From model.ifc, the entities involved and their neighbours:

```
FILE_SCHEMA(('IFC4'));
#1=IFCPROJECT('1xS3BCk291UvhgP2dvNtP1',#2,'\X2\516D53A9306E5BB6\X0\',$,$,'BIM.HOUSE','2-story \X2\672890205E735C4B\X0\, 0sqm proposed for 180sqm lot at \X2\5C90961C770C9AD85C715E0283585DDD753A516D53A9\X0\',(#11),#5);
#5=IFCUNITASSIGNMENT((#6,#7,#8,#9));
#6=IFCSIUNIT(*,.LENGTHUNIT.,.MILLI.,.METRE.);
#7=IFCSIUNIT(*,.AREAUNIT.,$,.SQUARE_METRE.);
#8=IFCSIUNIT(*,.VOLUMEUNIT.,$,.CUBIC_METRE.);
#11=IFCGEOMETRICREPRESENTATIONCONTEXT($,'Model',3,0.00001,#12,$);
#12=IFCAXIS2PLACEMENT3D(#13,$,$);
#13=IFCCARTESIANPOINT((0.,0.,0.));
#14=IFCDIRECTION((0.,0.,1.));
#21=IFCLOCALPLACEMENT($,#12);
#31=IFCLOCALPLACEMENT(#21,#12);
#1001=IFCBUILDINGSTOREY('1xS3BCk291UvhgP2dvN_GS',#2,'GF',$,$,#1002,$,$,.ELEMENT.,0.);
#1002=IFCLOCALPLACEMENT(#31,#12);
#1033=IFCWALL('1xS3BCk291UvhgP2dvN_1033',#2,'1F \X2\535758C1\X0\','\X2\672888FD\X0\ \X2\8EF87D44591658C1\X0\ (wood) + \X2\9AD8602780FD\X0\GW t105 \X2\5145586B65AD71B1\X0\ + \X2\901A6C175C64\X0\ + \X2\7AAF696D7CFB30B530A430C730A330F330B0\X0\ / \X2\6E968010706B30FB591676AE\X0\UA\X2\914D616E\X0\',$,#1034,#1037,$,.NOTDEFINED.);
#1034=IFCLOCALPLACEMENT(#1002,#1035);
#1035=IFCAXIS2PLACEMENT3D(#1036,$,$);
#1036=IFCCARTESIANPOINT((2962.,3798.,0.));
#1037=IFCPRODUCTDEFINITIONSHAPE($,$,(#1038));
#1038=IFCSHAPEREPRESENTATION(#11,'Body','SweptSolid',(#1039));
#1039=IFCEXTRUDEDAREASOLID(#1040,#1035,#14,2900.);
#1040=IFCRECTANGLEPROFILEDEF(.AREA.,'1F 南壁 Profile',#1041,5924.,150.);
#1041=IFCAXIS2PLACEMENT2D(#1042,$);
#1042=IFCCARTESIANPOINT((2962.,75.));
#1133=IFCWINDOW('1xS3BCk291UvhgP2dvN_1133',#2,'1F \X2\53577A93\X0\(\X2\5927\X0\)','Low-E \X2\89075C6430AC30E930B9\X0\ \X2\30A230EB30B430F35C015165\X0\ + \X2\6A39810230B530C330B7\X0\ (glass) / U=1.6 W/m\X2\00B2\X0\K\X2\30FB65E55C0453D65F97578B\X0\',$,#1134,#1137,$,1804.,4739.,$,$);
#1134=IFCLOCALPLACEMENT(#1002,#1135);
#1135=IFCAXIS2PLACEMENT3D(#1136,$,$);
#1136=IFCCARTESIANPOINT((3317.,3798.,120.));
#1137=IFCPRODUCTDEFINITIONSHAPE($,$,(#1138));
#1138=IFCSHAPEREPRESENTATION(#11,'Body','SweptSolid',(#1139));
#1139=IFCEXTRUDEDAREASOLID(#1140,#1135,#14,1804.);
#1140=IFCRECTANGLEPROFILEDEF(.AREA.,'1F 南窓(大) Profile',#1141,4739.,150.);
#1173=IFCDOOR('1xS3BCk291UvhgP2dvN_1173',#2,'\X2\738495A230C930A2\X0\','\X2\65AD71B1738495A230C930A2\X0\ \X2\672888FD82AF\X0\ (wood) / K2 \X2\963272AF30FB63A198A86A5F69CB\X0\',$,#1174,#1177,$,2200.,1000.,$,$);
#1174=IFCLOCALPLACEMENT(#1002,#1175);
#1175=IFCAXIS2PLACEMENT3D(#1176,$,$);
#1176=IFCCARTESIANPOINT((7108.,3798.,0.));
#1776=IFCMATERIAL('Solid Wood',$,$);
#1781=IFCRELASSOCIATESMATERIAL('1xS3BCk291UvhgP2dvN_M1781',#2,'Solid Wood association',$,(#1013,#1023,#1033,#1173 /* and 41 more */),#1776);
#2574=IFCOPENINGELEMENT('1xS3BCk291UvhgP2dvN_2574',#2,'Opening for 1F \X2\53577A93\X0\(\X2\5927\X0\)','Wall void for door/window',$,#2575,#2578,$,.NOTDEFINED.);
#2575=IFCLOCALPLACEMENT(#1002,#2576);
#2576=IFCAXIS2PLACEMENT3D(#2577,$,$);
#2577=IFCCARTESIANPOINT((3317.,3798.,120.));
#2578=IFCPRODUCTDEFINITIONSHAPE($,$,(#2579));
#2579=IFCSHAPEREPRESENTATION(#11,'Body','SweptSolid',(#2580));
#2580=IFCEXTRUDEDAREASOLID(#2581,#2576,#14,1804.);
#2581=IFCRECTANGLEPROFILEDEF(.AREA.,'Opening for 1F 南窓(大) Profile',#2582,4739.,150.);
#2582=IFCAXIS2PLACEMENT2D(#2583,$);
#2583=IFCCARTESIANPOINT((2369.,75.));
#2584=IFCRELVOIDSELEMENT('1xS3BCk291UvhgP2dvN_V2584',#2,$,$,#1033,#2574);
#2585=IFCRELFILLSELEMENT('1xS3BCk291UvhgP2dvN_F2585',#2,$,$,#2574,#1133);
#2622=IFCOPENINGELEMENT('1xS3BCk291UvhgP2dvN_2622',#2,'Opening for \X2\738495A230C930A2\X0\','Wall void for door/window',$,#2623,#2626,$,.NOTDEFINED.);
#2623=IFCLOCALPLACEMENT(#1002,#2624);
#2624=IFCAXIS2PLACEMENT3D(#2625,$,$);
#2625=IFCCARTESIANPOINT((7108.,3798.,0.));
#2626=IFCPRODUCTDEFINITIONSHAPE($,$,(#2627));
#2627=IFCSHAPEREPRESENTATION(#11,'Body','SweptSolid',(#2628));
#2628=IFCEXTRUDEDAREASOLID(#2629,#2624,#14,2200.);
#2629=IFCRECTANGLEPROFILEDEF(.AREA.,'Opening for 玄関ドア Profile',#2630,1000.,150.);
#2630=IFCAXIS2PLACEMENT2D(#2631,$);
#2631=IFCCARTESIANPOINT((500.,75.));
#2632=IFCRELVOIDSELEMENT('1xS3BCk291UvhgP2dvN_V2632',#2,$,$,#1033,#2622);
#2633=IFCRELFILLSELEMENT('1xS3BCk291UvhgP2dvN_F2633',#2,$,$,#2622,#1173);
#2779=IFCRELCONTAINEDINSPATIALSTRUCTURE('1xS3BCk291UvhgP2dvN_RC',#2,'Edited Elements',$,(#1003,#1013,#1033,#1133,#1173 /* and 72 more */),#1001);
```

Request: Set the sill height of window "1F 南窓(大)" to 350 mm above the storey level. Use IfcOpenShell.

```python
import numpy as np
import ifcopenshell
import ifcopenshell.api.geometry
import ifcopenshell.geom
import ifcopenshell.util.element
import ifcopenshell.util.placement
import ifcopenshell.util.shape
import ifcopenshell.util.unit

model = ifcopenshell.open("model.ifc")
unit_scale = ifcopenshell.util.unit.calculate_unit_scale(model)

window = model.by_guid("1xS3BCk291UvhgP2dvN_1133")
opening = window.FillsVoids[0].RelatingOpeningElement
storey = ifcopenshell.util.element.get_container(window, ifc_class="IfcBuildingStorey")
level = ifcopenshell.util.placement.get_local_placement(storey.ObjectPlacement)[2, 3]

# The opening's origin need not be at the sill, so measure its lowest point.
shape = ifcopenshell.geom.create_shape(ifcopenshell.geom.settings(), opening)
bottom = ifcopenshell.util.shape.get_shape_bottom_elevation(shape, shape.geometry) / unit_scale
dz = level + 350.0 - bottom

shift = np.array([0.0, 0.0, dz])
# The window is not placed relative to its opening, so move both.
for product in (opening, window):
    matrix = ifcopenshell.util.placement.get_local_placement(product.ObjectPlacement)
    matrix[:3, 3] += shift
    ifcopenshell.api.geometry.edit_object_placement(model, product=product, matrix=matrix, is_si=False)

print(f"moved by {dz * unit_scale:+.3f} m")

model.write("model-out.ifc")
```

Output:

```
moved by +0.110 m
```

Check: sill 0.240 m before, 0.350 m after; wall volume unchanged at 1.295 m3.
